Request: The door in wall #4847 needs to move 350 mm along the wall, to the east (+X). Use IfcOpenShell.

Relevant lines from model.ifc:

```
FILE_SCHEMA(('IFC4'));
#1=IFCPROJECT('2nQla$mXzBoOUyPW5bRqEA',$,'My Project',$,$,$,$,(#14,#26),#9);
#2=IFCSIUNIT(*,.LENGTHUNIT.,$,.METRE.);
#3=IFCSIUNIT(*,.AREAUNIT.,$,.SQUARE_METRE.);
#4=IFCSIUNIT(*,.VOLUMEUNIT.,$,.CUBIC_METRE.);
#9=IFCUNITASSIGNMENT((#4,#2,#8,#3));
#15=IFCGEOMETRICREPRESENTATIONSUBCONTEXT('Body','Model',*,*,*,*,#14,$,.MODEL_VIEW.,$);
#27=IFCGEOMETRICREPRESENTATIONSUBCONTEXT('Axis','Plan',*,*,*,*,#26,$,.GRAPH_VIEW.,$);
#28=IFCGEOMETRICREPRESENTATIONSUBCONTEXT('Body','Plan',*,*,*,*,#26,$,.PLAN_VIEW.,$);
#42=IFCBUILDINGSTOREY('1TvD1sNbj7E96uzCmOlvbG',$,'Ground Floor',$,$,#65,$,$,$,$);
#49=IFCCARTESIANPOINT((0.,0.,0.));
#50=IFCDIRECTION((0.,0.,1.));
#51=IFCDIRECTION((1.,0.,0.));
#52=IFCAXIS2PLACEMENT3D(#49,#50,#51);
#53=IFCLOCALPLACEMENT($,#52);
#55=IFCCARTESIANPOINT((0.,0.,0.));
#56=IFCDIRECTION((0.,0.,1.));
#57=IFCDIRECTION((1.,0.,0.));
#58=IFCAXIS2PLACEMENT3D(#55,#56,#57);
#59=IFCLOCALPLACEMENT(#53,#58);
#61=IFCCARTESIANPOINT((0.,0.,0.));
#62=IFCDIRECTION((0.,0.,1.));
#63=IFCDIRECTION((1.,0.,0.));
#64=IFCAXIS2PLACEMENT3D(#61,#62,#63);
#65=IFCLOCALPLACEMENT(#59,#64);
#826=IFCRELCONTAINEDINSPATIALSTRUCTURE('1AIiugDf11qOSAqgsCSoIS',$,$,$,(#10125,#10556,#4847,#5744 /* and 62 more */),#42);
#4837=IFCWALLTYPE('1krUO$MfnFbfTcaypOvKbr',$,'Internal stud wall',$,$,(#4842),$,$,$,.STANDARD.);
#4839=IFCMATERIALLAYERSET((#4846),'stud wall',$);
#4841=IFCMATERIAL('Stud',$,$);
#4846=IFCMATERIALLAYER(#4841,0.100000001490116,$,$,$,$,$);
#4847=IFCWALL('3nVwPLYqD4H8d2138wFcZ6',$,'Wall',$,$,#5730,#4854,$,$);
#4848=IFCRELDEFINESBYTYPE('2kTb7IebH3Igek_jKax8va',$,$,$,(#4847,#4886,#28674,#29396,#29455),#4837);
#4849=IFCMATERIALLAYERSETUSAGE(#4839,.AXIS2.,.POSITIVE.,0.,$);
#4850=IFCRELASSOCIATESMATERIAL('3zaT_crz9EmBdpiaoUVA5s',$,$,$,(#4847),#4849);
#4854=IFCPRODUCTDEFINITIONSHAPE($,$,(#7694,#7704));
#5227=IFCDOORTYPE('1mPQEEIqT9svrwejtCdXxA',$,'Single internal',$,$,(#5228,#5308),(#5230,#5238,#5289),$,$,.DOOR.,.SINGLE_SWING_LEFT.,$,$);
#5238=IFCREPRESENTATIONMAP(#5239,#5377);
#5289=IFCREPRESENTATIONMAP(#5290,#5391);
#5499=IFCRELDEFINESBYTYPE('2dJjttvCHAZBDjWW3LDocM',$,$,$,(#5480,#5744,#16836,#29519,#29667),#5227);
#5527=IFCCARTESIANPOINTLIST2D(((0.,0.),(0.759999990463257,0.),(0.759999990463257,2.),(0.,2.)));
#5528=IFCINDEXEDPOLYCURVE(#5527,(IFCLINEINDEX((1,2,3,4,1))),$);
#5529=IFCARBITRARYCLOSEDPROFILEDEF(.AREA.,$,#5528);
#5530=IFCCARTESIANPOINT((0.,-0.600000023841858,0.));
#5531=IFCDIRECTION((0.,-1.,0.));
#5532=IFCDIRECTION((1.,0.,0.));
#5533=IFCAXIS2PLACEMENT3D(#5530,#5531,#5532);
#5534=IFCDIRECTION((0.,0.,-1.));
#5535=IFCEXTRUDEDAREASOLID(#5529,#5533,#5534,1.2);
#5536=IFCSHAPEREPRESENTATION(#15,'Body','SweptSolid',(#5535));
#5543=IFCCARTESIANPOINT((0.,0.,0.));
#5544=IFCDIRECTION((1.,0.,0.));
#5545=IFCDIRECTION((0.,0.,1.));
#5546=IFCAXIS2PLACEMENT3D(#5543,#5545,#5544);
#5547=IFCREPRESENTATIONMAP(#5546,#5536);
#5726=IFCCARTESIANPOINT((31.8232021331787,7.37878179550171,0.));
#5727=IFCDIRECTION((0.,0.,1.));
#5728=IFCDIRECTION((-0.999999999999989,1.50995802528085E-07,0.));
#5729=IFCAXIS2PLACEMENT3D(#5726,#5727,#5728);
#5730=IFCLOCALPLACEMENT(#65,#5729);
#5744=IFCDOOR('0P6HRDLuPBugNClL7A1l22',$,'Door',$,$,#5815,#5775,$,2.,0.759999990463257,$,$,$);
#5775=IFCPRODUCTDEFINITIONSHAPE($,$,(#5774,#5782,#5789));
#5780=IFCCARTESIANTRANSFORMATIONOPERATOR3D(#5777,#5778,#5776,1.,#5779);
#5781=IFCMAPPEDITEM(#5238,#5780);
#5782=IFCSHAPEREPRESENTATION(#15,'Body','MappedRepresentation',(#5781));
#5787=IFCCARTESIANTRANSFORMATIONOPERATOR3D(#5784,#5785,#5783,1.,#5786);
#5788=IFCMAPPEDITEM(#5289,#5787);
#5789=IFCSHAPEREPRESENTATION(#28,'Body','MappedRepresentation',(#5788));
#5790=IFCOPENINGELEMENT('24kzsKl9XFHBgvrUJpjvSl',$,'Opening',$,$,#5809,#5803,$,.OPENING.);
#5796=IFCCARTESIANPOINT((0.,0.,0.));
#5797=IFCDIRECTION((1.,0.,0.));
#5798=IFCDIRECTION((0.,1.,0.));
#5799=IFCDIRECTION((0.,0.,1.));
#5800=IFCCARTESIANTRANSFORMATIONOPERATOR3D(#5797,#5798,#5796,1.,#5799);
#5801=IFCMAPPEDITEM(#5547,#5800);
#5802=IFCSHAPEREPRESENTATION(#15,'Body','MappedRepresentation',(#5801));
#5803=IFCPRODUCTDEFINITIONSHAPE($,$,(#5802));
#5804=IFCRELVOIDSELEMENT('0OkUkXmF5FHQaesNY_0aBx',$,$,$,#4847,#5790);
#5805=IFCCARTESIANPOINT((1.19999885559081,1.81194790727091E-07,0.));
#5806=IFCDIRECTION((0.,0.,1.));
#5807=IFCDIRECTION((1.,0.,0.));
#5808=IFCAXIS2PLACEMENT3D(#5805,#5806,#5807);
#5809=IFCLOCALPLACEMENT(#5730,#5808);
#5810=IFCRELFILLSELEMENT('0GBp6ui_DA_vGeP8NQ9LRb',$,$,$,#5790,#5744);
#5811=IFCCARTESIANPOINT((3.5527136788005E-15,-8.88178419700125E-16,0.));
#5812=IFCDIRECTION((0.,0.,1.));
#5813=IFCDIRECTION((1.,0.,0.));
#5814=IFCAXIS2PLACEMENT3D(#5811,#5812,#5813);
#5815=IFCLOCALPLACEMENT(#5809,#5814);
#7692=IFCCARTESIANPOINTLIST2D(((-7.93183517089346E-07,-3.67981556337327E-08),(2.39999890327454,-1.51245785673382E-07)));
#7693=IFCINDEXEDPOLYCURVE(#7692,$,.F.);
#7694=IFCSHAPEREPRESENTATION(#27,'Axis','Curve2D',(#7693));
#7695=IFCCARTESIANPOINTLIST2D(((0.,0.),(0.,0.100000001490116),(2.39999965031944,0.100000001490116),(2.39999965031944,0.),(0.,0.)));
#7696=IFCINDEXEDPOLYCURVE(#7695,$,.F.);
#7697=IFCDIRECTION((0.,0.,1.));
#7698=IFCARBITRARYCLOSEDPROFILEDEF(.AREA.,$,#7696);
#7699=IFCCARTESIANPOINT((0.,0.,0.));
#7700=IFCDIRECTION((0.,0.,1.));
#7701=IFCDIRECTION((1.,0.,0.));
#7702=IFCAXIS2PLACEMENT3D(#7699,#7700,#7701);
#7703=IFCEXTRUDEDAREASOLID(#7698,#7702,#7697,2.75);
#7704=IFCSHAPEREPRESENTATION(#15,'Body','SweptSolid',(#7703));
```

```python
import ifcopenshell
import ifcopenshell.api.geometry
import ifcopenshell.util.placement
import ifcopenshell.util.unit

model = ifcopenshell.open("model.ifc")
unit_scale = ifcopenshell.util.unit.calculate_unit_scale(model)

door = model.by_guid("0P6HRDLuPBugNClL7A1l22")
opening = door.FillsVoids[0].RelatingOpeningElement
wall = opening.VoidsElements[0].RelatingBuildingElement

wall_matrix = ifcopenshell.util.placement.get_local_placement(wall.ObjectPlacement)
shift = wall_matrix[:3, 0] * -0.35 / unit_scale
before = ifcopenshell.util.placement.get_local_placement(door.ObjectPlacement)[:3, 3].copy()

# The door is placed relative to its opening, so it follows when the opening moves.
matrix = ifcopenshell.util.placement.get_local_placement(opening.ObjectPlacement)
matrix[:3, 3] += shift
ifcopenshell.api.geometry.edit_object_placement(
    model, product=opening, matrix=matrix, is_si=False, should_transform_children=True
)

after = ifcopenshell.util.placement.get_local_placement(door.ObjectPlacement)[:3, 3]
print("door moved by", (after - before).round(3) + 0.0)

model.write("model-out.ifc")
```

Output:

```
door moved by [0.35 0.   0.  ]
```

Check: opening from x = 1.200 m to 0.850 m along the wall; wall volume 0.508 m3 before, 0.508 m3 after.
